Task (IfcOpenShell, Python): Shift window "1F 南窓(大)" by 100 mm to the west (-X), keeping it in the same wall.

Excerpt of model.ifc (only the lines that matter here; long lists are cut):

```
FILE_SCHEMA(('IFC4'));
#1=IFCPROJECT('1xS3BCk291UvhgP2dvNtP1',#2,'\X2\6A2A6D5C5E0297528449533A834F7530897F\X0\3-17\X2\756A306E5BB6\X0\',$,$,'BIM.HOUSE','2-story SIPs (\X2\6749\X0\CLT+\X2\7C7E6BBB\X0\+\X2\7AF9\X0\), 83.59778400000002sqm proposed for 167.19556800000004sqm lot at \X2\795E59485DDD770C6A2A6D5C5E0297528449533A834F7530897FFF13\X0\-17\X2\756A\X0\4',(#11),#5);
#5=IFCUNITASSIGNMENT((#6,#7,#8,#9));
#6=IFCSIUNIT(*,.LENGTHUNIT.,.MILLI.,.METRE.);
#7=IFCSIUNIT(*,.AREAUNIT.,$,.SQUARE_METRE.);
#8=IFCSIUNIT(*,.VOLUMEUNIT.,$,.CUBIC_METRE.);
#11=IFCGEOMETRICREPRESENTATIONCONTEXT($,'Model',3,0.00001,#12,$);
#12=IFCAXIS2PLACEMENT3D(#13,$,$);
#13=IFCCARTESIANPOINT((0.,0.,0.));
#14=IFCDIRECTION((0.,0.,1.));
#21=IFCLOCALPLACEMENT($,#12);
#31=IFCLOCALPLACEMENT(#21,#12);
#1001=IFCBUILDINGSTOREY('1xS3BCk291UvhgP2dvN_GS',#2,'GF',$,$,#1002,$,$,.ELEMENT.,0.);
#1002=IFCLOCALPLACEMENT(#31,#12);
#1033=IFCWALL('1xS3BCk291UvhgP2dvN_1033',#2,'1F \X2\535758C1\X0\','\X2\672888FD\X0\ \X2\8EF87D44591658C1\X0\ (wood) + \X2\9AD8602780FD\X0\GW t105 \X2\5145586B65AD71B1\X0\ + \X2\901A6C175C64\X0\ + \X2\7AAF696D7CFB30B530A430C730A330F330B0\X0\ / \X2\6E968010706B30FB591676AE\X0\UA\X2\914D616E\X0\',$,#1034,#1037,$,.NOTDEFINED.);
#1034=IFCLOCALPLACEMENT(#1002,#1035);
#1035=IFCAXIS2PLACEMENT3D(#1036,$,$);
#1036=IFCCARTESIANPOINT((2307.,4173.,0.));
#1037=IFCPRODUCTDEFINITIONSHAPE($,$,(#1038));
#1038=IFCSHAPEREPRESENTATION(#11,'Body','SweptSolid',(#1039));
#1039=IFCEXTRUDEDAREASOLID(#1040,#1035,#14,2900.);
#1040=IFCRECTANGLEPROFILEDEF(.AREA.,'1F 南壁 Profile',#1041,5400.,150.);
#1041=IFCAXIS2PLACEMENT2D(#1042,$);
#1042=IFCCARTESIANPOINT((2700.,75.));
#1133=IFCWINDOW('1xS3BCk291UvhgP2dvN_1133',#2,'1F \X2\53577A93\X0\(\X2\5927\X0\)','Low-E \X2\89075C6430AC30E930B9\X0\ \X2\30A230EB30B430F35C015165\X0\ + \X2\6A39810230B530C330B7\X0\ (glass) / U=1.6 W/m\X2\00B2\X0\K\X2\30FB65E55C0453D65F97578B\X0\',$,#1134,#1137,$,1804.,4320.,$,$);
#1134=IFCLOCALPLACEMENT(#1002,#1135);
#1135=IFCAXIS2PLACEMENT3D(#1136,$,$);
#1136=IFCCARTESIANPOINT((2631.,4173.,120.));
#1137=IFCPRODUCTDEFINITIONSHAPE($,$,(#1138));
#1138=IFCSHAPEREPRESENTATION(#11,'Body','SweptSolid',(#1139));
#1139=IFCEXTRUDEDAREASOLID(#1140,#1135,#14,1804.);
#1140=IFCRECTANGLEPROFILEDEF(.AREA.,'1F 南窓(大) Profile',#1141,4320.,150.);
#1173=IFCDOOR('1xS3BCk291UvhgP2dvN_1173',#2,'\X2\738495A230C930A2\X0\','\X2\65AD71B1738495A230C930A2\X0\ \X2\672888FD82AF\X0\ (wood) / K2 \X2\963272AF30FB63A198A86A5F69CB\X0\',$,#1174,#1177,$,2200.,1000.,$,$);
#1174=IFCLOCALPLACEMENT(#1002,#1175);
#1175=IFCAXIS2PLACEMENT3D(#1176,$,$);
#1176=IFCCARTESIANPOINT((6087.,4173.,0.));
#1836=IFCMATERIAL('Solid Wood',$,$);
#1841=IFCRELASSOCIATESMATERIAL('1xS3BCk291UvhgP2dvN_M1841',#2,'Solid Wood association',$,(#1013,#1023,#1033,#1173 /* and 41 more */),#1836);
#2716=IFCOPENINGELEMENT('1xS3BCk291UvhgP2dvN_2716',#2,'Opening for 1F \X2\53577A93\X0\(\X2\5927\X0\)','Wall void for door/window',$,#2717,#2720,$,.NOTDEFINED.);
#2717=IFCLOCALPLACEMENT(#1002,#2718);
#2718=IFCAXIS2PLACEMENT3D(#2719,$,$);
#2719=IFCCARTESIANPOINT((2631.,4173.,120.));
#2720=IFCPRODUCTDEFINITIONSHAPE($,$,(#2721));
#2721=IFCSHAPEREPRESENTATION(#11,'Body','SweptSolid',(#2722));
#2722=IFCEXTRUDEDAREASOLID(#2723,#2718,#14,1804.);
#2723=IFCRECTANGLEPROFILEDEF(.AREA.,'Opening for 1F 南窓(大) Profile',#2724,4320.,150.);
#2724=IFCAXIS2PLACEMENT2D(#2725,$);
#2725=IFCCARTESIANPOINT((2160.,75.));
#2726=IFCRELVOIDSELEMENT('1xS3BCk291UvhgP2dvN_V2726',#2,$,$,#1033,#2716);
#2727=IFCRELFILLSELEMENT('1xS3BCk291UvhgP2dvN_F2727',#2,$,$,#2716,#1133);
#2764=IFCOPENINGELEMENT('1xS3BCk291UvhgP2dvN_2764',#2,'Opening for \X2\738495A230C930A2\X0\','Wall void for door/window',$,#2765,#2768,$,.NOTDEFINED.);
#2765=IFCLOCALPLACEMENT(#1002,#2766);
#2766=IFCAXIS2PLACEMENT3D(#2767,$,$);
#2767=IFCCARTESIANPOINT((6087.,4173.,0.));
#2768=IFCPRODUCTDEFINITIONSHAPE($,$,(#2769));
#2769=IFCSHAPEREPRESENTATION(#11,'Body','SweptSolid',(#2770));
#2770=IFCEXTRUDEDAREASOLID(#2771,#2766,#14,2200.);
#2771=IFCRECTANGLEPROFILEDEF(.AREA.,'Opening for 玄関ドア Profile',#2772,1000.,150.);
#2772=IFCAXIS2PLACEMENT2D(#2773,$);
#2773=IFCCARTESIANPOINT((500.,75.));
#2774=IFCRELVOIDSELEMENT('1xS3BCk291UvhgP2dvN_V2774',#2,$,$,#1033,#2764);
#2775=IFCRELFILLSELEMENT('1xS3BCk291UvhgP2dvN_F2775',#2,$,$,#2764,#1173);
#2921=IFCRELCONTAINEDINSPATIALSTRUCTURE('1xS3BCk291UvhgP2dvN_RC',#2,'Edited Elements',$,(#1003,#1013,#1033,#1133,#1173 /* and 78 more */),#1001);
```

```python
import ifcopenshell
import ifcopenshell.api.geometry
import ifcopenshell.util.placement

model = ifcopenshell.open("model.ifc")

window = model.by_guid("1xS3BCk291UvhgP2dvN_1133")
opening = window.FillsVoids[0].RelatingOpeningElement
wall = opening.VoidsElements[0].RelatingBuildingElement

wall_matrix = ifcopenshell.util.placement.get_local_placement(wall.ObjectPlacement)
shift = wall_matrix[:3, 0] * -100.0
before = ifcopenshell.util.placement.get_local_placement(window.ObjectPlacement)[:3, 3].copy()

# The window is not placed relative to its opening, so move both.
for product in (opening, window):
    matrix = ifcopenshell.util.placement.get_local_placement(product.ObjectPlacement)
    matrix[:3, 3] += shift
    ifcopenshell.api.geometry.edit_object_placement(model, product=product, matrix=matrix, is_si=False)

after = ifcopenshell.util.placement.get_local_placement(window.ObjectPlacement)[:3, 3]
print("window moved by", (after - before).round(3) + 0.0)

model.write("model_updated.ifc")
```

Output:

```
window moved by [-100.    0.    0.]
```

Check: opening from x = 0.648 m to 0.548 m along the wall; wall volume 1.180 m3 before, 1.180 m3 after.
